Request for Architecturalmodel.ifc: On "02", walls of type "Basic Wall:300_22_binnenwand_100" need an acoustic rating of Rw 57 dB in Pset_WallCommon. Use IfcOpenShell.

First a look at what the model holds.

```python
import ifcopenshell
import ifcopenshell.util.element

model = ifcopenshell.open("Architecturalmodel.ifc")
print(model.schema)
storey = next(s for s in model.by_type("IfcBuildingStorey") if s.Name == "02")
walls = [e for e in ifcopenshell.util.element.get_decomposition(storey) if e.is_a("IfcWall")]
seen = {}
for e in walls:
    element_type = ifcopenshell.util.element.get_type(e)
    key = (element_type.Name if element_type != e and element_type else None, ifcopenshell.util.element.get_pset(e, "Pset_WallCommon", "AcousticRating"))
    seen[key] = seen.get(key, 0) + 1
for (name, value), count in sorted(seen.items(), key=str):
    print(count, "x", name, "|", value)
```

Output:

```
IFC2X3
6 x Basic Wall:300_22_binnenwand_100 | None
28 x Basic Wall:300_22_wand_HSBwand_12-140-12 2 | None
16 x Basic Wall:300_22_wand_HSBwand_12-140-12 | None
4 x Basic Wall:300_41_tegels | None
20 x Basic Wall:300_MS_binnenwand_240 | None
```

```python
import ifcopenshell
import ifcopenshell.api.pset
import ifcopenshell.util.element

model = ifcopenshell.open("Architecturalmodel.ifc")

storey = next(s for s in model.by_type("IfcBuildingStorey") if s.Name == "02")
walls = [e for e in ifcopenshell.util.element.get_decomposition(storey) if e.is_a("IfcWall")]

count = 0
for e in walls:
    element_type = ifcopenshell.util.element.get_type(e)
    if element_type in (None, e) or element_type.Name != "Basic Wall:300_22_binnenwand_100":
        continue
    # add_pset returns the element's existing set when there is one.
    pset = ifcopenshell.api.pset.add_pset(model, product=e, name="Pset_WallCommon")
    ifcopenshell.api.pset.edit_pset(model, pset=pset, properties={"AcousticRating": "Rw 57 dB"})
    count += 1

print(count, "walls updated")

model.write("Architecturalmodel_updated.ifc")
```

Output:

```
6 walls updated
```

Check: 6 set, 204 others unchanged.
